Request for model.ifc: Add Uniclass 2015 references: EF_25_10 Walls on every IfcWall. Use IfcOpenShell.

First a look at what the model holds.

```python
import ifcopenshell

model = ifcopenshell.open("model.ifc")
print(model.schema)
print("classifications:", [c.Name for c in model.by_type("IfcClassification")])
for ifc_class in ("IfcDoor", "IfcRoof", "IfcStair", "IfcWall", "IfcWindow"):
    print(ifc_class, len(model.by_type(ifc_class)))
```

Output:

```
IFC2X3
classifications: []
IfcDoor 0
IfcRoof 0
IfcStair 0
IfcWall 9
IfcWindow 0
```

```python
import ifcopenshell
import ifcopenshell.api.classification

model = ifcopenshell.open("model.ifc")

# IFC2X3 requires Source and Edition and has no link from the project to the system.
system = model.create_entity("IfcClassification", Source="NBS", Edition="2015", Name="Uniclass 2015")

codes = {
    "IfcWall": ("EF_25_10", "Walls"),
}
for ifc_class, (code, name) in codes.items():
    products = model.by_type(ifc_class)
    ifcopenshell.api.classification.add_reference(
        model, products=products, classification=system, identification=code, name=name
    )
    print(code, len(products))

model.write("model_updated.ifc")
```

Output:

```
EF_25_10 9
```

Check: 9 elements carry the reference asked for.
